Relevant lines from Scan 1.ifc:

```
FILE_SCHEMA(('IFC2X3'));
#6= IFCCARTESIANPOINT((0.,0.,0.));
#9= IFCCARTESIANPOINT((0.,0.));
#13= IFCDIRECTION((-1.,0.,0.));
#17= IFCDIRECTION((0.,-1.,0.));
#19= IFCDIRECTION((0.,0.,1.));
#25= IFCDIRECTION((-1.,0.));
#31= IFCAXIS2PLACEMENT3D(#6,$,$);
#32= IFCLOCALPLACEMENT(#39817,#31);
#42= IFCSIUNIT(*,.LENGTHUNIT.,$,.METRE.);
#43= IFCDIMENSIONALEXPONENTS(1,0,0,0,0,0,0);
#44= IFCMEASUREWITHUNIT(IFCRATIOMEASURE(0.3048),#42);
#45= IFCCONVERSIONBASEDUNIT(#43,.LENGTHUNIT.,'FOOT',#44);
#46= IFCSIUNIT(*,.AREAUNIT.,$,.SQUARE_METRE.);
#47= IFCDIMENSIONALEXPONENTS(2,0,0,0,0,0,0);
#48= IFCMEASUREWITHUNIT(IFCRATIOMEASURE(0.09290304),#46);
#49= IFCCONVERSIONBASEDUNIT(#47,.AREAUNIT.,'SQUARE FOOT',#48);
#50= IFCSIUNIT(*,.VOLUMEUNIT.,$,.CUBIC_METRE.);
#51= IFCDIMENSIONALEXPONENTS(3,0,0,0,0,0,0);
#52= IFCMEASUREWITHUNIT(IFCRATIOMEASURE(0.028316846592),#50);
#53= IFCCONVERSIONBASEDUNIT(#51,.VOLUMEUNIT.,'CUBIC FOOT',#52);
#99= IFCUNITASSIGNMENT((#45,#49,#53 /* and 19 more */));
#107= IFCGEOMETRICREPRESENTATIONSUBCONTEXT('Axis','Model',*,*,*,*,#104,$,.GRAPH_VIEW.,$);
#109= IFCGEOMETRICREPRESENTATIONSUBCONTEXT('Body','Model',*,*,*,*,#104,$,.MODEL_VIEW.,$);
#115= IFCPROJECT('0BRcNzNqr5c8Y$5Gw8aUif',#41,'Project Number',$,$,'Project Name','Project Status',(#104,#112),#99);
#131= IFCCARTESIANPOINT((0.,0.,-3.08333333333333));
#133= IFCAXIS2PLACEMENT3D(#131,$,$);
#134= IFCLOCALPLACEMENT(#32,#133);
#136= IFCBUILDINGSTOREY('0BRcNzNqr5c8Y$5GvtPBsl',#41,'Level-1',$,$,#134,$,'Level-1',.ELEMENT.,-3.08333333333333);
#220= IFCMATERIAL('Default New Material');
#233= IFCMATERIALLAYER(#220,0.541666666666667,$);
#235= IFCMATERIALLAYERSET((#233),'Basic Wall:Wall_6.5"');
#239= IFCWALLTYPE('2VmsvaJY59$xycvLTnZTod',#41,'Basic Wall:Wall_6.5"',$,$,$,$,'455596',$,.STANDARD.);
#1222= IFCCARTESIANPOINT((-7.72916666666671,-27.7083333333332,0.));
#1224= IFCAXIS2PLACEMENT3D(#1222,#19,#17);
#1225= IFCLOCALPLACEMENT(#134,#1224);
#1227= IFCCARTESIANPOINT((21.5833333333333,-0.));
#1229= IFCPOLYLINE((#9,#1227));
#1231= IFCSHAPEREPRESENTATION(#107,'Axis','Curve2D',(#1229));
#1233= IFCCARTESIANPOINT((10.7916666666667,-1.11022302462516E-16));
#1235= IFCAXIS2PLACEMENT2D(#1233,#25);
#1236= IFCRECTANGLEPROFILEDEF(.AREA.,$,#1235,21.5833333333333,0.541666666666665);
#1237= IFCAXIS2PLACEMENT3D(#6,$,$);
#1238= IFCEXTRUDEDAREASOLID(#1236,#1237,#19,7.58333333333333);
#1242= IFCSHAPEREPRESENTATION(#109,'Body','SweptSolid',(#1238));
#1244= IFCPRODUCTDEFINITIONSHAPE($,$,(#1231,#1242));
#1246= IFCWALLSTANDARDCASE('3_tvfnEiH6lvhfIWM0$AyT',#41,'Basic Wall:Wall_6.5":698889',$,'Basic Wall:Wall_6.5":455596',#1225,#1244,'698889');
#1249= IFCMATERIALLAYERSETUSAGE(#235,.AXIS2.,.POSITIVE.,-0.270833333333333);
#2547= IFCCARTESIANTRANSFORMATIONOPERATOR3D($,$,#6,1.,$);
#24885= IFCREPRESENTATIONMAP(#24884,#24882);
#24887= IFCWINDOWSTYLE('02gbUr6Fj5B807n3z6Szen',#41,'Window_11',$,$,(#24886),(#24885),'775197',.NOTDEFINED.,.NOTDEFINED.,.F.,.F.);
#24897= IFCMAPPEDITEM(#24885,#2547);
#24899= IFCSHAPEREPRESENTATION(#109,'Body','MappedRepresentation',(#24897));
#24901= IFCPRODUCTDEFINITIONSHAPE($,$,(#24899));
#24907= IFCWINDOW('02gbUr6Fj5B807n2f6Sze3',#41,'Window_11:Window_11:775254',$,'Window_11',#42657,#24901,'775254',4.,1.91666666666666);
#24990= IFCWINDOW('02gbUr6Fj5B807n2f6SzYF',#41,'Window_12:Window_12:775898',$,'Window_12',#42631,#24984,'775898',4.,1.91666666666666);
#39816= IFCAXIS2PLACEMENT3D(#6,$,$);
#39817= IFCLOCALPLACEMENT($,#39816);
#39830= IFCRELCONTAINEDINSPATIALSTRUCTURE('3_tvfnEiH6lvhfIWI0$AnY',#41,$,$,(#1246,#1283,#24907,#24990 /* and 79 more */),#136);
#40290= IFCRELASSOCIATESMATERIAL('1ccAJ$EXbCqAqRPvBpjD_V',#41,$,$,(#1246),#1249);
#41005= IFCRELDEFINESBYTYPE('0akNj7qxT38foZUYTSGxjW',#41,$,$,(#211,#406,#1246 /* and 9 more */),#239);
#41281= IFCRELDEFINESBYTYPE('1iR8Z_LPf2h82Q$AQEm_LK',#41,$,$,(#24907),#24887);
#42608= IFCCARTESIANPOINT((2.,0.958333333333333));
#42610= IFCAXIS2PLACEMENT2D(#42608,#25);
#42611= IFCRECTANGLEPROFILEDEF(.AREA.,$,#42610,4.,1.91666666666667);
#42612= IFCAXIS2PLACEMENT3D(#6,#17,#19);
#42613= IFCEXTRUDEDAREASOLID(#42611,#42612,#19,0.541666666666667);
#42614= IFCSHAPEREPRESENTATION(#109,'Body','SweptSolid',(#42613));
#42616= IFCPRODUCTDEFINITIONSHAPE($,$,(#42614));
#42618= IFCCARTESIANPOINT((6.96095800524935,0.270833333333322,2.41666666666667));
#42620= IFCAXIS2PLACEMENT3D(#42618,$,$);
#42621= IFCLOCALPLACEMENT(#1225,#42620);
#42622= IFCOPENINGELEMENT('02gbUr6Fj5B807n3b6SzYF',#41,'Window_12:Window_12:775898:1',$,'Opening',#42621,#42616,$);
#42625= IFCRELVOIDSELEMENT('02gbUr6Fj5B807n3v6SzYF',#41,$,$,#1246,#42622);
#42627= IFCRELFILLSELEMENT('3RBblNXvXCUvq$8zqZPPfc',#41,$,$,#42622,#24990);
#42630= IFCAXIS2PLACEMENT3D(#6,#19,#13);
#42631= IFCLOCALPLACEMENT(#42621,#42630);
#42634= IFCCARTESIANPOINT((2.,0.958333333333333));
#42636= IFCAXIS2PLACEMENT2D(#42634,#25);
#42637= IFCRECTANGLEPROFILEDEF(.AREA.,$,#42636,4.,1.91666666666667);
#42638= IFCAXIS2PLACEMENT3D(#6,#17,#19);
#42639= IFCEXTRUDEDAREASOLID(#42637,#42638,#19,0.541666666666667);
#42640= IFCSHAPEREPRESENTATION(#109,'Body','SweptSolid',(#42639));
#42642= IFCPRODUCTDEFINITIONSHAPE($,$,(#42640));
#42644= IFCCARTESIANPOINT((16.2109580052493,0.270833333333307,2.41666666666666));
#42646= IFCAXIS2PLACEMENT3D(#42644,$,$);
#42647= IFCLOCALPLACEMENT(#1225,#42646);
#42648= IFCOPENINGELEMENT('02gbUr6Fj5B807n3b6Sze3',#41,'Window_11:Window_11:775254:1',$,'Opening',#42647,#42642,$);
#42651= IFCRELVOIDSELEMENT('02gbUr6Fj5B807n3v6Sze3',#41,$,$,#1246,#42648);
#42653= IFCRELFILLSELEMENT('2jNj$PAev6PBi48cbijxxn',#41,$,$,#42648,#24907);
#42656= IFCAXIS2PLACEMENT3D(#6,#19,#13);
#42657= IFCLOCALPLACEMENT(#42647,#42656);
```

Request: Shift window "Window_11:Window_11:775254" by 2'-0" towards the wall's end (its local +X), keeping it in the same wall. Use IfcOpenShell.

```python
import ifcopenshell
import ifcopenshell.api.geometry
import ifcopenshell.util.placement
import ifcopenshell.util.unit

model = ifcopenshell.open("Scan 1.ifc")
unit_scale = ifcopenshell.util.unit.calculate_unit_scale(model)

window = model.by_guid("02gbUr6Fj5B807n2f6Sze3")
opening = window.FillsVoids[0].RelatingOpeningElement
wall = opening.VoidsElements[0].RelatingBuildingElement

wall_matrix = ifcopenshell.util.placement.get_local_placement(wall.ObjectPlacement)
shift = wall_matrix[:3, 0] * 24 * 0.0254 / unit_scale
before = ifcopenshell.util.placement.get_local_placement(window.ObjectPlacement)[:3, 3].copy()

# The window is placed relative to its opening, so it follows when the opening moves.
matrix = ifcopenshell.util.placement.get_local_placement(opening.ObjectPlacement)
matrix[:3, 3] += shift
ifcopenshell.api.geometry.edit_object_placement(
    model, product=opening, matrix=matrix, is_si=False, should_transform_children=True
)

after = ifcopenshell.util.placement.get_local_placement(window.ObjectPlacement)[:3, 3]
print("window moved by", (after - before).round(3) + 0.0)

model.write("Scan 1-out.ifc")
```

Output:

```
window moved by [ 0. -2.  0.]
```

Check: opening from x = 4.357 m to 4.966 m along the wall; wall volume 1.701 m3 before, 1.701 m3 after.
